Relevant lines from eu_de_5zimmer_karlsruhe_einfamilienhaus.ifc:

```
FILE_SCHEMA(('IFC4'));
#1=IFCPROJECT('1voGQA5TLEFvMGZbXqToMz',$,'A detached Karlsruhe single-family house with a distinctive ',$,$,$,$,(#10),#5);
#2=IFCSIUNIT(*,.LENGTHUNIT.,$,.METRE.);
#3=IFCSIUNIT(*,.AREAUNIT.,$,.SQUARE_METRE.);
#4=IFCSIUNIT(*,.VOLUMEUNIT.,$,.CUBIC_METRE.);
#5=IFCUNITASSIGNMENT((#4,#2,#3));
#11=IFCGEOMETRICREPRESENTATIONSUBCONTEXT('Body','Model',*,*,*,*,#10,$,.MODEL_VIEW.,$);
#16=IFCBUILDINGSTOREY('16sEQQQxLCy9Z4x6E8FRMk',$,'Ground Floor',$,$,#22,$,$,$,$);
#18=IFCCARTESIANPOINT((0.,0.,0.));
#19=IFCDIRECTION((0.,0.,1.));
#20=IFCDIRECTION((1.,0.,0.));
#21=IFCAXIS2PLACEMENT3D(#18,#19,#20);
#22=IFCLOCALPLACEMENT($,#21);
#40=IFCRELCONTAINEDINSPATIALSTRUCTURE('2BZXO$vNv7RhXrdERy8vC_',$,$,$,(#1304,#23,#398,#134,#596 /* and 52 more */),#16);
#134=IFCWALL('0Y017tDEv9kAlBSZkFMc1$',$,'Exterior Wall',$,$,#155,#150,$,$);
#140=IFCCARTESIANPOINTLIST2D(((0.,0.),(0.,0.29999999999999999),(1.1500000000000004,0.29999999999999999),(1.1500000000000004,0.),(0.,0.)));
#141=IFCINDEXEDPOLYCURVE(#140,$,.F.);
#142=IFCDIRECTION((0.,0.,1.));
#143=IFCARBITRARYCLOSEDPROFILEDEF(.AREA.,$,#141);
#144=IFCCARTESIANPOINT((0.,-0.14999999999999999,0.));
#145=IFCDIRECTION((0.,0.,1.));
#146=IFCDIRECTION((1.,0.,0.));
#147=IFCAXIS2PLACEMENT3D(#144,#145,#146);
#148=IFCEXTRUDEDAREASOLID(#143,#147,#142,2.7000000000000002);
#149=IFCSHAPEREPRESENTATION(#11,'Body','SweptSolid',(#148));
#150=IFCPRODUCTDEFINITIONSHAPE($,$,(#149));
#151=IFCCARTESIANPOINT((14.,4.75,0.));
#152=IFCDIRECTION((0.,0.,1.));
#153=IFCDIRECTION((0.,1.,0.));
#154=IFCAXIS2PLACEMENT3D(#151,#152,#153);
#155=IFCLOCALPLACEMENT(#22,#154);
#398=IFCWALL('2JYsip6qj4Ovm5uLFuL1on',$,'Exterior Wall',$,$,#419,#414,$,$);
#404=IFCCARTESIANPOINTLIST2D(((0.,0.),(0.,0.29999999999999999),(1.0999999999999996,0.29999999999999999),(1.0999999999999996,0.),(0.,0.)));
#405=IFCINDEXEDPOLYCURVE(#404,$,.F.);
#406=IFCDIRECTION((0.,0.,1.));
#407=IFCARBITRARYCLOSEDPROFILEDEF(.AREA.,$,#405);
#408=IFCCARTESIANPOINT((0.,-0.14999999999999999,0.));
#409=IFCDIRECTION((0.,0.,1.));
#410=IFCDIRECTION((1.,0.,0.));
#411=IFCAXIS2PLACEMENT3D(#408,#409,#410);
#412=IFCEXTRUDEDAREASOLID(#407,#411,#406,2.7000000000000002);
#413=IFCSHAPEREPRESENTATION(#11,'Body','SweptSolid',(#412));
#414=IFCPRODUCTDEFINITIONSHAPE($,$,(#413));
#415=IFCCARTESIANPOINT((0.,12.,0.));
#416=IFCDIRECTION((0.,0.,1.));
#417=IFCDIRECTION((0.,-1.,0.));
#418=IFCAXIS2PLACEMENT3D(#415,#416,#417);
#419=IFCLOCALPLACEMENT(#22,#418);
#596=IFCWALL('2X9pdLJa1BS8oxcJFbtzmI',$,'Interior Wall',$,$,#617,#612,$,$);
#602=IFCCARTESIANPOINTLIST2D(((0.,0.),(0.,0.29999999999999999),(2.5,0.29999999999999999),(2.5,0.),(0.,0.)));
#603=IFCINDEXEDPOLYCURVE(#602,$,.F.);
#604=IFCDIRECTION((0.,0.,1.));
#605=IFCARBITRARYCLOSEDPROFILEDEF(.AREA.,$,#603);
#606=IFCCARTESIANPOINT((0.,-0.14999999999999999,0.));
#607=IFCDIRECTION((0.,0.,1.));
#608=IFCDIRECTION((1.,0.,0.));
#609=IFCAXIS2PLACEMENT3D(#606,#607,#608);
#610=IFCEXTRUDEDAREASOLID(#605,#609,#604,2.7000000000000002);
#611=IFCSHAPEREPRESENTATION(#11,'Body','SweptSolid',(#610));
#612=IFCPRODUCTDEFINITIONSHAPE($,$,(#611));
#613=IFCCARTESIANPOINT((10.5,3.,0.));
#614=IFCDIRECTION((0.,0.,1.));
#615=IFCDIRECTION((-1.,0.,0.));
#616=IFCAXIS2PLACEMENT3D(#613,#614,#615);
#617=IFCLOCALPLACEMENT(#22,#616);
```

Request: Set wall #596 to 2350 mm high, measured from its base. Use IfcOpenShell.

```python
import ifcopenshell
import ifcopenshell.geom
import ifcopenshell.util.representation
import ifcopenshell.util.shape
import ifcopenshell.util.unit

model = ifcopenshell.open("eu_de_5zimmer_karlsruhe_einfamilienhaus.ifc")
unit_scale = ifcopenshell.util.unit.calculate_unit_scale(model)
settings = ifcopenshell.geom.settings()


def volume(element):
    """Net volume in cubic metres, openings subtracted."""
    shape = ifcopenshell.geom.create_shape(settings, element)
    return ifcopenshell.util.shape.get_volume(shape.geometry)


wall = model.by_id(596)
before = volume(wall)

body = ifcopenshell.util.representation.get_representation(wall, "Model", "Body")
solid = body.Items[0]
old_height = solid.Depth
solid.Depth = 2.35 / unit_scale
after = volume(wall)

print(f"height {old_height:g} -> {solid.Depth:g}, volume {before:.3f} -> {after:.3f} m3")

model.write("eu_de_5zimmer_karlsruhe_einfamilienhaus_rev.ifc")
```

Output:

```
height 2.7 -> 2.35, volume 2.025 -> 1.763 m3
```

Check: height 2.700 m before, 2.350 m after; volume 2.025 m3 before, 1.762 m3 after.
